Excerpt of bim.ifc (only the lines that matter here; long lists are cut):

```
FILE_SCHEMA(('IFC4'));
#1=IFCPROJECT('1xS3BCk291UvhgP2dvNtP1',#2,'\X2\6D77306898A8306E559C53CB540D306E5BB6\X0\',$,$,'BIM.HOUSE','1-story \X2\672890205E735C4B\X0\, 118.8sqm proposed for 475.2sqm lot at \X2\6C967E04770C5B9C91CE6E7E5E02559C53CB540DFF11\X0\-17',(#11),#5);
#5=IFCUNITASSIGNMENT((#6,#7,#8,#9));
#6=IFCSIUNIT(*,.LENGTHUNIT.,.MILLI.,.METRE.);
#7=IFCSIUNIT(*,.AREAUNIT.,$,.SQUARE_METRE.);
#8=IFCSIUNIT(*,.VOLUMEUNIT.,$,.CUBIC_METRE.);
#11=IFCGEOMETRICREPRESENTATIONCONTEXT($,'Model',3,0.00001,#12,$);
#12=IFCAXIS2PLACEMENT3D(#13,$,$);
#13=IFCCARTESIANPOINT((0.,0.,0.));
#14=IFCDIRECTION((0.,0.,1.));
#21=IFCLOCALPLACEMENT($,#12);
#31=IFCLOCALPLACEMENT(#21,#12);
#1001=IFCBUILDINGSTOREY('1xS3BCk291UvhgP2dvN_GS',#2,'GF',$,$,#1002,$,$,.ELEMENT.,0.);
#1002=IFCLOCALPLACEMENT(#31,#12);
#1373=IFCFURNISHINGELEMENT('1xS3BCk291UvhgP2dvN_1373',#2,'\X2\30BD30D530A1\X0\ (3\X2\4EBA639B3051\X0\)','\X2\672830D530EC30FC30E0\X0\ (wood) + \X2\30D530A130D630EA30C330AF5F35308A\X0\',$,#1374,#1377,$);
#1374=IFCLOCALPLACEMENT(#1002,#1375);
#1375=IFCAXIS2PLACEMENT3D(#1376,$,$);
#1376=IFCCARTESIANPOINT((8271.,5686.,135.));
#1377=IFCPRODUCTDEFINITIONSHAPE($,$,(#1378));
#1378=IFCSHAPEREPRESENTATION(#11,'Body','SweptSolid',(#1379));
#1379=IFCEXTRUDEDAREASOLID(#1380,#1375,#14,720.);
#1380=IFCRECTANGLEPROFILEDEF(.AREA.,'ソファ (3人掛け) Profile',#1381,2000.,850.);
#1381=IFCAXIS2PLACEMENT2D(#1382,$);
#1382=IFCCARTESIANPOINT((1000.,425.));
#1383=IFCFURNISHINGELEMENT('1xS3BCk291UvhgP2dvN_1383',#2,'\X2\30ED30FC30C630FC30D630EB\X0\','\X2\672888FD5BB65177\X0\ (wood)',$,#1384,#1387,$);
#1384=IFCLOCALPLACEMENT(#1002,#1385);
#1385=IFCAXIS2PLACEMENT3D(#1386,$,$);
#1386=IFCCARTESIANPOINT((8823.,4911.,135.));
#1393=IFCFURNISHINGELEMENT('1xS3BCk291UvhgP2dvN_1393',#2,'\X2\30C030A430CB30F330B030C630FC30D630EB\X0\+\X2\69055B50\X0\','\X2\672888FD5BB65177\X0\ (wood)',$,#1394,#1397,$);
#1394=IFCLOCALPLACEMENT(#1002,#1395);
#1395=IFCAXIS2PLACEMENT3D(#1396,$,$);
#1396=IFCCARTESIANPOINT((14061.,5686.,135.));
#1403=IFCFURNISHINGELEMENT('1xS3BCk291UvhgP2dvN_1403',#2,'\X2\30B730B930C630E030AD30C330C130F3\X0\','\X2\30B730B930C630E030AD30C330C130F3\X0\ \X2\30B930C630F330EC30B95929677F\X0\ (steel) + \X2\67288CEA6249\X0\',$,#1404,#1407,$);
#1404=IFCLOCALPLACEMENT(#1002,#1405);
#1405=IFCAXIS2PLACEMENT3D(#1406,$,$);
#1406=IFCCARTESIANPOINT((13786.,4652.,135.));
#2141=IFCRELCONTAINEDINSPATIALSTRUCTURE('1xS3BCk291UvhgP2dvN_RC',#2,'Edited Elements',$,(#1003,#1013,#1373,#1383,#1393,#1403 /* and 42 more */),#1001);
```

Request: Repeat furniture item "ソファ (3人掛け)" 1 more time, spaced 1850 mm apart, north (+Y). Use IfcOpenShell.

```python
import numpy as np
import ifcopenshell
import ifcopenshell.api.geometry
import ifcopenshell.api.root
import ifcopenshell.util.element
import ifcopenshell.util.placement

model = ifcopenshell.open("bim.ifc")


def reuse_history(source, copy):
    """copy_class also copies each property set's owner history, people and application; keep the originals."""
    for rel in copy.IsDefinedBy:
        if rel.is_a("IfcRelDefinesByProperties") and (history := rel.RelatingPropertyDefinition.OwnerHistory):
            rel.RelatingPropertyDefinition.OwnerHistory = source.OwnerHistory
            ifcopenshell.util.element.remove_deep2(model, history)


source = model.by_guid("1xS3BCk291UvhgP2dvN_1373")
base = ifcopenshell.util.placement.get_local_placement(source.ObjectPlacement)
step = np.array([0.0, 1.0, 0.0]) * 1850.0

for i in range(1, 2):
    copy = ifcopenshell.api.root.copy_class(model, product=source)
    copy.Representation = ifcopenshell.util.element.copy_deep(
        model, source.Representation, exclude=["IfcGeometricRepresentationContext", "IfcRepresentationMap"]
    )
    reuse_history(source, copy)
    matrix = base.copy()
    matrix[:3, 3] += i * step
    print("added at", matrix[:3, 3].round(3) + 0.0)
    ifcopenshell.api.geometry.edit_object_placement(model, product=copy, matrix=matrix, is_si=False)

model.write("bim_rev.ifc")
```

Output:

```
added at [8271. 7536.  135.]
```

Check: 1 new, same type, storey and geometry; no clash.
